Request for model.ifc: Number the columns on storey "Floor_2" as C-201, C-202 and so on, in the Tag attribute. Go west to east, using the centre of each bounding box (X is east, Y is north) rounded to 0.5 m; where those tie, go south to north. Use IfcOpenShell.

First a look at what the model holds.

```python
import ifcopenshell
import ifcopenshell.util.element
import ifcopenshell.util.placement

model = ifcopenshell.open("model.ifc")
print(model.schema)
storey = next(s for s in model.by_type("IfcBuildingStorey") if s.Name == "Floor_2")
columns = [e for e in ifcopenshell.util.element.get_decomposition(storey) if e.is_a("IfcColumn")]
for e in sorted(columns, key=lambda e: e.id()):
    origin = ifcopenshell.util.placement.get_local_placement(e.ObjectPlacement)[:3, 3]
    print(e.id(), e.Tag, e.Name, origin.round(2) + 0.0, sep=" | ")
```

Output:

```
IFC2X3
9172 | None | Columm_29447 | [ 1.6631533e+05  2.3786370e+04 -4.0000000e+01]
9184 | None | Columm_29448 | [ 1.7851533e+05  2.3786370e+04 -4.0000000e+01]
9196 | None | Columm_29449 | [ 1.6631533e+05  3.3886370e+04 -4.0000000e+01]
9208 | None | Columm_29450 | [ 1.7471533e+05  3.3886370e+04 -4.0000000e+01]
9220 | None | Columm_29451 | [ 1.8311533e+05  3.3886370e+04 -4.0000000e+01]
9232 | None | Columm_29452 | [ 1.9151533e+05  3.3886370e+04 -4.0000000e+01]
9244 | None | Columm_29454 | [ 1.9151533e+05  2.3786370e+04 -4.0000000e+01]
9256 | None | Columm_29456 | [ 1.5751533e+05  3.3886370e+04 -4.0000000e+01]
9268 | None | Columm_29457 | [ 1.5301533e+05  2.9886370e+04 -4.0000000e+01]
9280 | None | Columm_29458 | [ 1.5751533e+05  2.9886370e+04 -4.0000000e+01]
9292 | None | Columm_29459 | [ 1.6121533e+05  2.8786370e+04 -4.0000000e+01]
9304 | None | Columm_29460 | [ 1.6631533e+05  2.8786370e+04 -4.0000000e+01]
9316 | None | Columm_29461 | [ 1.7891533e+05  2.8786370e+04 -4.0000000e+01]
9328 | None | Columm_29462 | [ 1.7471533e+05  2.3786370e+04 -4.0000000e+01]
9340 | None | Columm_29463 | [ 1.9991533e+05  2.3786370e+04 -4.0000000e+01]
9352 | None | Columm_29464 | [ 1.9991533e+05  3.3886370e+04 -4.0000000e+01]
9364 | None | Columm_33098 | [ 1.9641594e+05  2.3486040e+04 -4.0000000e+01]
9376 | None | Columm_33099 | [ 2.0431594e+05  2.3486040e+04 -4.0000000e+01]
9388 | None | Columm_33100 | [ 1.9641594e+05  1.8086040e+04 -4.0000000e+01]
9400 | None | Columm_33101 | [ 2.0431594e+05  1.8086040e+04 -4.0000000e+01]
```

```python
import ifcopenshell
import ifcopenshell.geom
import ifcopenshell.util.element
import ifcopenshell.util.shape

model = ifcopenshell.open("model.ifc")
settings = ifcopenshell.geom.settings()
settings.set("use-world-coords", True)


def centre(element):
    shape = ifcopenshell.geom.create_shape(settings, element)
    return ifcopenshell.util.shape.get_bbox_centroid(shape.geometry)


storey = next(s for s in model.by_type("IfcBuildingStorey") if s.Name == "Floor_2")
columns = [e for e in ifcopenshell.util.element.get_decomposition(storey) if e.is_a("IfcColumn")]

# Insertion points can sit at a corner or the storey origin, so sort by the geometry (in metres).
centres = {e: centre(e) for e in columns}
columns.sort(key=lambda e: (round(centres[e][0] / 0.5), centres[e][1]))

for i, e in enumerate(columns, start=1):
    number = f"C-2{i:02d}"
    e.Tag = number
    print(e.id(), number)

model.write("model-out.ifc")
```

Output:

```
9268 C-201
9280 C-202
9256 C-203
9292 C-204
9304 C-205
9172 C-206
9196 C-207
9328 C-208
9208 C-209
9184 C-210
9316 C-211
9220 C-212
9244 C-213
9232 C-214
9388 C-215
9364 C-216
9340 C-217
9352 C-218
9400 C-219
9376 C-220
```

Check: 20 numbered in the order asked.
